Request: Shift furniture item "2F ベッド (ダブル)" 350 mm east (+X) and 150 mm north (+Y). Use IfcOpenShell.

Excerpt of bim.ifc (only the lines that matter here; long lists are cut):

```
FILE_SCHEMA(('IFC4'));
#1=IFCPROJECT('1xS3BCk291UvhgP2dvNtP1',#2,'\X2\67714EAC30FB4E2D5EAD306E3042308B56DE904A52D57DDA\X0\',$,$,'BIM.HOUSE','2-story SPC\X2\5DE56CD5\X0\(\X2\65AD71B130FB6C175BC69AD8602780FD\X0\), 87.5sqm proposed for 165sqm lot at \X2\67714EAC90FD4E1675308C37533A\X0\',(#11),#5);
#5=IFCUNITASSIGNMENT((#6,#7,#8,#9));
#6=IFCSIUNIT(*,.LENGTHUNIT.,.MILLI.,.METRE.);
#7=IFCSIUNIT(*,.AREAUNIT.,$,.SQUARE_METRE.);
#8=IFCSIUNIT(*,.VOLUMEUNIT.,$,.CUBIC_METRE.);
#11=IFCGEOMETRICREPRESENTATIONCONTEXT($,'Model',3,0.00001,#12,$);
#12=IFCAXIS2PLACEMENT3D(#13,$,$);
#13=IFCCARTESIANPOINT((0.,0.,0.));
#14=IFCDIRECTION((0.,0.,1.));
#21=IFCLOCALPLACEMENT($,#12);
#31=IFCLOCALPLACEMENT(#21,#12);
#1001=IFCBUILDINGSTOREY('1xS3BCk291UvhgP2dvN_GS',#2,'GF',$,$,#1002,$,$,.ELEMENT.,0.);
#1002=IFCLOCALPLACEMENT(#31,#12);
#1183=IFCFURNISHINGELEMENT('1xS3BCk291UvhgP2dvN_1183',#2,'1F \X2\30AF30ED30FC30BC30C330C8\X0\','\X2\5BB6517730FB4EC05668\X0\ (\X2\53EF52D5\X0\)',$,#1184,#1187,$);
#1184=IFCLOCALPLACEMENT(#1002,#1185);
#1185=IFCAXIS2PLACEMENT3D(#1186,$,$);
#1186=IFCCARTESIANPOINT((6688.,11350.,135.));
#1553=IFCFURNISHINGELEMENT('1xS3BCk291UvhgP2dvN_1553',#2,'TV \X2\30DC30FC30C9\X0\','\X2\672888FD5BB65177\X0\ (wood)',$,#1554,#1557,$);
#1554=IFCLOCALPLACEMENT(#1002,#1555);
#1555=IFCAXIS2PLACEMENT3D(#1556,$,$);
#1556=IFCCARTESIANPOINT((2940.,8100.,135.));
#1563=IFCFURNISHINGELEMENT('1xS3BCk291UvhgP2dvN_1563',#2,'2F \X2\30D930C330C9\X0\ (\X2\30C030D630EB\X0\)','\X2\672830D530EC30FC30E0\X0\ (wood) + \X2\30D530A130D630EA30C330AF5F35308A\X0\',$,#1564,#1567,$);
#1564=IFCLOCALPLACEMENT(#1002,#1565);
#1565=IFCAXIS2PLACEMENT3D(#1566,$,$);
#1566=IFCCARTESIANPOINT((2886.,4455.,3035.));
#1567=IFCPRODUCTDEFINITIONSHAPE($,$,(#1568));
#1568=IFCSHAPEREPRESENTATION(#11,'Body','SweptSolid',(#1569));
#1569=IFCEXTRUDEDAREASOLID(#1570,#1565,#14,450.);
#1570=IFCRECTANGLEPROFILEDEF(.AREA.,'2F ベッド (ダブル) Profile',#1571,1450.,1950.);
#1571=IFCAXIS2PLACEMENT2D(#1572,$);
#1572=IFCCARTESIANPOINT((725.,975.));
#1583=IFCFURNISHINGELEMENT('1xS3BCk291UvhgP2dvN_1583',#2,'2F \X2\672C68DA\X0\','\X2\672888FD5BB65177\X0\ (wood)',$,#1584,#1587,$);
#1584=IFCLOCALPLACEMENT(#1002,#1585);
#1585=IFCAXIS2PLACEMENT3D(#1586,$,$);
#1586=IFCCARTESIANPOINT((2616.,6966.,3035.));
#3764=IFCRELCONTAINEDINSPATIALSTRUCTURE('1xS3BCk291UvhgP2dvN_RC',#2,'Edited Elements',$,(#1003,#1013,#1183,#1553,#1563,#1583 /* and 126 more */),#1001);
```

```python
import ifcopenshell
import ifcopenshell.api.geometry
import ifcopenshell.util.placement
import ifcopenshell.util.unit

model = ifcopenshell.open("bim.ifc")
unit_scale = ifcopenshell.util.unit.calculate_unit_scale(model)

item = model.by_guid("1xS3BCk291UvhgP2dvN_1563")
matrix = ifcopenshell.util.placement.get_local_placement(item.ObjectPlacement)
matrix[0, 3] += 0.35 / unit_scale
matrix[1, 3] += 0.15 / unit_scale
ifcopenshell.api.geometry.edit_object_placement(model, product=item, matrix=matrix, is_si=False)

print(ifcopenshell.util.placement.get_local_placement(item.ObjectPlacement).round(3) + 0.0)

model.write("bim_rev.ifc")
```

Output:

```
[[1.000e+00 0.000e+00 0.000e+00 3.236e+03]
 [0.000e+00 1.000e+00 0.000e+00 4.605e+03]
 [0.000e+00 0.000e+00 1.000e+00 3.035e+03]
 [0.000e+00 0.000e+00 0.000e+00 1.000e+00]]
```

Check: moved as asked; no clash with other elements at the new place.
